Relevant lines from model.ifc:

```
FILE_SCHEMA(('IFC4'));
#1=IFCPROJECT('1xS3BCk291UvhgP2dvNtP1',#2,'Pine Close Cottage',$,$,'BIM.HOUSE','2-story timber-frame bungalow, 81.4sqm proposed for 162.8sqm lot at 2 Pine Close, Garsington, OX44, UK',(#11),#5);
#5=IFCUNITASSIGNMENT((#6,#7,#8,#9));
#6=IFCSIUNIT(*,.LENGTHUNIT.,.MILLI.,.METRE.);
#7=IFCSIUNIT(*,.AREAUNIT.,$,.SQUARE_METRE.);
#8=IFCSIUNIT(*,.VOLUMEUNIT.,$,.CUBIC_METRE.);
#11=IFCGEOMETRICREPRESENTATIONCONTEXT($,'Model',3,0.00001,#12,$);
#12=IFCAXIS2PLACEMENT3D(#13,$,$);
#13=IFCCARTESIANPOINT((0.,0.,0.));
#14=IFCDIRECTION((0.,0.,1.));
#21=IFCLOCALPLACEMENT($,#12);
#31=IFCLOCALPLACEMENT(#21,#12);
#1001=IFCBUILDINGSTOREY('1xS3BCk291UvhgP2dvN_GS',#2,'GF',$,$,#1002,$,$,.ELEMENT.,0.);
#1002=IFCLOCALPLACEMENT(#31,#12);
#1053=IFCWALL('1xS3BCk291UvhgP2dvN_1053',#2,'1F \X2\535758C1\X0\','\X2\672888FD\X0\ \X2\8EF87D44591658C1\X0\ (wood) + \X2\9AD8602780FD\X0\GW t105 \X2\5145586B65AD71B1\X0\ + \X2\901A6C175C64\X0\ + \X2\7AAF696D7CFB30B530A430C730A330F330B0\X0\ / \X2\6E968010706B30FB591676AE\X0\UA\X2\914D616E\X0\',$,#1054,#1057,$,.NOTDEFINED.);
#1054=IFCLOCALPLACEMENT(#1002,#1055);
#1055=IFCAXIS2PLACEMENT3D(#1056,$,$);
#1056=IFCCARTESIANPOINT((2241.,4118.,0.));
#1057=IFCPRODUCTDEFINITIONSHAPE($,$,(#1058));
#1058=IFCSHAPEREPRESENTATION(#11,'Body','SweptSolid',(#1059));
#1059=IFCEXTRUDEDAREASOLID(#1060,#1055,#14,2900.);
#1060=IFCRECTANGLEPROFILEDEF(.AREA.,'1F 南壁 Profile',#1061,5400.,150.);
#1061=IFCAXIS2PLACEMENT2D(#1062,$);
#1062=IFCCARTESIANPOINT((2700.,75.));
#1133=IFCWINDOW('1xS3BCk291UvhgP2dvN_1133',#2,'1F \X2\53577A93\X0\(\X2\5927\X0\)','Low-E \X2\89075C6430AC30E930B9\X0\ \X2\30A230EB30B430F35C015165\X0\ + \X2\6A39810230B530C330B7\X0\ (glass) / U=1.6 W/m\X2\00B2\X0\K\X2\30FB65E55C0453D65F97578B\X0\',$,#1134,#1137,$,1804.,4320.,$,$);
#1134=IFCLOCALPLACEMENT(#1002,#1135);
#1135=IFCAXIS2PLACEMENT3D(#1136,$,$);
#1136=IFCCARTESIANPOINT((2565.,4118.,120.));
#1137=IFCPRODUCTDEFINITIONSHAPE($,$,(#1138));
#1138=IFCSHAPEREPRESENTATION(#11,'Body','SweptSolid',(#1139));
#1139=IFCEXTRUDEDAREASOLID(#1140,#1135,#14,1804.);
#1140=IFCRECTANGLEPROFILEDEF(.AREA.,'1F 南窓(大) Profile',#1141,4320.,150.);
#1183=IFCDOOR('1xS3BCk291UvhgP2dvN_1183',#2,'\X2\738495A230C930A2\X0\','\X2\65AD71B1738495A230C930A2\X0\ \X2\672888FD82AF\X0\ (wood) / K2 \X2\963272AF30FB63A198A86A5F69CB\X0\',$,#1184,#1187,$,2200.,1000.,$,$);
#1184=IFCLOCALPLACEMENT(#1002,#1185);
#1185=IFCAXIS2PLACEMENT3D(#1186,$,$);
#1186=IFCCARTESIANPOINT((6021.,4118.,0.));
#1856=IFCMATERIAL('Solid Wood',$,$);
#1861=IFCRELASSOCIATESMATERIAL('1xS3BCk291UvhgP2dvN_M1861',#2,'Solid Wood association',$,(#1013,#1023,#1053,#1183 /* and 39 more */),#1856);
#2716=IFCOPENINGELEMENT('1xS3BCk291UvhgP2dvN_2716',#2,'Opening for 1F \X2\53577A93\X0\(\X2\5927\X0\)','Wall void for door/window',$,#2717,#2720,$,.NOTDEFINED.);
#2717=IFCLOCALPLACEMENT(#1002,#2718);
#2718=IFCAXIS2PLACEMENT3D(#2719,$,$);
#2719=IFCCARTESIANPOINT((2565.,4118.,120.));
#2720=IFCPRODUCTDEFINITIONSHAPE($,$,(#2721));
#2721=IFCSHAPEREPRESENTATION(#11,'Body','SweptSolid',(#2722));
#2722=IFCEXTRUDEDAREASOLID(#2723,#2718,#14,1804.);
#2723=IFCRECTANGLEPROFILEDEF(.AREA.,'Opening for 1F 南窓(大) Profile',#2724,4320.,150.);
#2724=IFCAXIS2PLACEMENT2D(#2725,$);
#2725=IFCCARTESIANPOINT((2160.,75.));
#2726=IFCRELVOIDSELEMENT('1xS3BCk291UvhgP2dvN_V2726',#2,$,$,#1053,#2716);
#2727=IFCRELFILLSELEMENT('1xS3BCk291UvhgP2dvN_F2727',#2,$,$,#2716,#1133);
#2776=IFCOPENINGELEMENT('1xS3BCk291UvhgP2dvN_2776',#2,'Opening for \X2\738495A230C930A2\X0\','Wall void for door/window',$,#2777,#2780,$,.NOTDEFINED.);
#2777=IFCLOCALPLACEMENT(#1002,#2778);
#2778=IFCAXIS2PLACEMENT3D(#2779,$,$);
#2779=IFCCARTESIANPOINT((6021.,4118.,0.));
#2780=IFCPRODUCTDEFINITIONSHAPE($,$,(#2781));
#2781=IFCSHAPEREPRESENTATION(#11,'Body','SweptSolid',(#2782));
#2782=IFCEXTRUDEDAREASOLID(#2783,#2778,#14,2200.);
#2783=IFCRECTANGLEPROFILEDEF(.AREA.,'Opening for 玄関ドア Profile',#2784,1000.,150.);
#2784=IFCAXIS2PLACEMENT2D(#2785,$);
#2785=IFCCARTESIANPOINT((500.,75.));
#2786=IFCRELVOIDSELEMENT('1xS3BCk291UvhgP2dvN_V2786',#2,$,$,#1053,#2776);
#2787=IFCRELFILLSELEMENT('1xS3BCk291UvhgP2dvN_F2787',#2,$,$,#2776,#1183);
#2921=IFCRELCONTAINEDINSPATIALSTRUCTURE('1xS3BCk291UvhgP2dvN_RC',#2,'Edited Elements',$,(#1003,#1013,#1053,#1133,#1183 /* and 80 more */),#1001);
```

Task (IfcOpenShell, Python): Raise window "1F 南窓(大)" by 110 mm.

```python
import numpy as np
import ifcopenshell
import ifcopenshell.api.geometry
import ifcopenshell.util.placement
import ifcopenshell.util.unit

model = ifcopenshell.open("model.ifc")
unit_scale = ifcopenshell.util.unit.calculate_unit_scale(model)

window = model.by_guid("1xS3BCk291UvhgP2dvN_1133")
opening = window.FillsVoids[0].RelatingOpeningElement
dz = 110.0

shift = np.array([0.0, 0.0, dz])
# The window is not placed relative to its opening, so move both.
for product in (opening, window):
    matrix = ifcopenshell.util.placement.get_local_placement(product.ObjectPlacement)
    matrix[:3, 3] += shift
    ifcopenshell.api.geometry.edit_object_placement(model, product=product, matrix=matrix, is_si=False)

print(f"moved by {dz * unit_scale:+.3f} m")

model.write("model-out.ifc")
```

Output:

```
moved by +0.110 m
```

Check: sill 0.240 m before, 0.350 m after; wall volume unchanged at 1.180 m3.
